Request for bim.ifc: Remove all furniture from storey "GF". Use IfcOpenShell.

First a look at what the model holds.

```python
import ifcopenshell
import ifcopenshell.util.element

model = ifcopenshell.open("bim.ifc")
print(model.schema)
storey = next(s for s in model.by_type("IfcBuildingStorey") if s.Name == "GF")
furniture = [e for e in ifcopenshell.util.element.get_decomposition(storey) if e.is_a("IfcFurnishingElement")]
seen = {}
for e in furniture:
    element_type = ifcopenshell.util.element.get_type(e)
    name = element_type.Name if element_type not in (None, e) else None
    seen[name] = seen.get(name, 0) + 1
for name, count in sorted(seen.items(), key=str):
    print(count, "x", name)
```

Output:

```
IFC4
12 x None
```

```python
import ifcopenshell
import ifcopenshell.api.root
import ifcopenshell.util.element

model = ifcopenshell.open("bim.ifc")

storey = next(s for s in model.by_type("IfcBuildingStorey") if s.Name == "GF")
furniture = [e for e in ifcopenshell.util.element.get_decomposition(storey) if e.is_a("IfcFurnishingElement")]

for e in furniture:
    ifcopenshell.api.root.remove_product(model, product=e)
print(len(furniture), "removed")

model.write("bim_rev.ifc")
```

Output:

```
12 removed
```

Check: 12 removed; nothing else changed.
